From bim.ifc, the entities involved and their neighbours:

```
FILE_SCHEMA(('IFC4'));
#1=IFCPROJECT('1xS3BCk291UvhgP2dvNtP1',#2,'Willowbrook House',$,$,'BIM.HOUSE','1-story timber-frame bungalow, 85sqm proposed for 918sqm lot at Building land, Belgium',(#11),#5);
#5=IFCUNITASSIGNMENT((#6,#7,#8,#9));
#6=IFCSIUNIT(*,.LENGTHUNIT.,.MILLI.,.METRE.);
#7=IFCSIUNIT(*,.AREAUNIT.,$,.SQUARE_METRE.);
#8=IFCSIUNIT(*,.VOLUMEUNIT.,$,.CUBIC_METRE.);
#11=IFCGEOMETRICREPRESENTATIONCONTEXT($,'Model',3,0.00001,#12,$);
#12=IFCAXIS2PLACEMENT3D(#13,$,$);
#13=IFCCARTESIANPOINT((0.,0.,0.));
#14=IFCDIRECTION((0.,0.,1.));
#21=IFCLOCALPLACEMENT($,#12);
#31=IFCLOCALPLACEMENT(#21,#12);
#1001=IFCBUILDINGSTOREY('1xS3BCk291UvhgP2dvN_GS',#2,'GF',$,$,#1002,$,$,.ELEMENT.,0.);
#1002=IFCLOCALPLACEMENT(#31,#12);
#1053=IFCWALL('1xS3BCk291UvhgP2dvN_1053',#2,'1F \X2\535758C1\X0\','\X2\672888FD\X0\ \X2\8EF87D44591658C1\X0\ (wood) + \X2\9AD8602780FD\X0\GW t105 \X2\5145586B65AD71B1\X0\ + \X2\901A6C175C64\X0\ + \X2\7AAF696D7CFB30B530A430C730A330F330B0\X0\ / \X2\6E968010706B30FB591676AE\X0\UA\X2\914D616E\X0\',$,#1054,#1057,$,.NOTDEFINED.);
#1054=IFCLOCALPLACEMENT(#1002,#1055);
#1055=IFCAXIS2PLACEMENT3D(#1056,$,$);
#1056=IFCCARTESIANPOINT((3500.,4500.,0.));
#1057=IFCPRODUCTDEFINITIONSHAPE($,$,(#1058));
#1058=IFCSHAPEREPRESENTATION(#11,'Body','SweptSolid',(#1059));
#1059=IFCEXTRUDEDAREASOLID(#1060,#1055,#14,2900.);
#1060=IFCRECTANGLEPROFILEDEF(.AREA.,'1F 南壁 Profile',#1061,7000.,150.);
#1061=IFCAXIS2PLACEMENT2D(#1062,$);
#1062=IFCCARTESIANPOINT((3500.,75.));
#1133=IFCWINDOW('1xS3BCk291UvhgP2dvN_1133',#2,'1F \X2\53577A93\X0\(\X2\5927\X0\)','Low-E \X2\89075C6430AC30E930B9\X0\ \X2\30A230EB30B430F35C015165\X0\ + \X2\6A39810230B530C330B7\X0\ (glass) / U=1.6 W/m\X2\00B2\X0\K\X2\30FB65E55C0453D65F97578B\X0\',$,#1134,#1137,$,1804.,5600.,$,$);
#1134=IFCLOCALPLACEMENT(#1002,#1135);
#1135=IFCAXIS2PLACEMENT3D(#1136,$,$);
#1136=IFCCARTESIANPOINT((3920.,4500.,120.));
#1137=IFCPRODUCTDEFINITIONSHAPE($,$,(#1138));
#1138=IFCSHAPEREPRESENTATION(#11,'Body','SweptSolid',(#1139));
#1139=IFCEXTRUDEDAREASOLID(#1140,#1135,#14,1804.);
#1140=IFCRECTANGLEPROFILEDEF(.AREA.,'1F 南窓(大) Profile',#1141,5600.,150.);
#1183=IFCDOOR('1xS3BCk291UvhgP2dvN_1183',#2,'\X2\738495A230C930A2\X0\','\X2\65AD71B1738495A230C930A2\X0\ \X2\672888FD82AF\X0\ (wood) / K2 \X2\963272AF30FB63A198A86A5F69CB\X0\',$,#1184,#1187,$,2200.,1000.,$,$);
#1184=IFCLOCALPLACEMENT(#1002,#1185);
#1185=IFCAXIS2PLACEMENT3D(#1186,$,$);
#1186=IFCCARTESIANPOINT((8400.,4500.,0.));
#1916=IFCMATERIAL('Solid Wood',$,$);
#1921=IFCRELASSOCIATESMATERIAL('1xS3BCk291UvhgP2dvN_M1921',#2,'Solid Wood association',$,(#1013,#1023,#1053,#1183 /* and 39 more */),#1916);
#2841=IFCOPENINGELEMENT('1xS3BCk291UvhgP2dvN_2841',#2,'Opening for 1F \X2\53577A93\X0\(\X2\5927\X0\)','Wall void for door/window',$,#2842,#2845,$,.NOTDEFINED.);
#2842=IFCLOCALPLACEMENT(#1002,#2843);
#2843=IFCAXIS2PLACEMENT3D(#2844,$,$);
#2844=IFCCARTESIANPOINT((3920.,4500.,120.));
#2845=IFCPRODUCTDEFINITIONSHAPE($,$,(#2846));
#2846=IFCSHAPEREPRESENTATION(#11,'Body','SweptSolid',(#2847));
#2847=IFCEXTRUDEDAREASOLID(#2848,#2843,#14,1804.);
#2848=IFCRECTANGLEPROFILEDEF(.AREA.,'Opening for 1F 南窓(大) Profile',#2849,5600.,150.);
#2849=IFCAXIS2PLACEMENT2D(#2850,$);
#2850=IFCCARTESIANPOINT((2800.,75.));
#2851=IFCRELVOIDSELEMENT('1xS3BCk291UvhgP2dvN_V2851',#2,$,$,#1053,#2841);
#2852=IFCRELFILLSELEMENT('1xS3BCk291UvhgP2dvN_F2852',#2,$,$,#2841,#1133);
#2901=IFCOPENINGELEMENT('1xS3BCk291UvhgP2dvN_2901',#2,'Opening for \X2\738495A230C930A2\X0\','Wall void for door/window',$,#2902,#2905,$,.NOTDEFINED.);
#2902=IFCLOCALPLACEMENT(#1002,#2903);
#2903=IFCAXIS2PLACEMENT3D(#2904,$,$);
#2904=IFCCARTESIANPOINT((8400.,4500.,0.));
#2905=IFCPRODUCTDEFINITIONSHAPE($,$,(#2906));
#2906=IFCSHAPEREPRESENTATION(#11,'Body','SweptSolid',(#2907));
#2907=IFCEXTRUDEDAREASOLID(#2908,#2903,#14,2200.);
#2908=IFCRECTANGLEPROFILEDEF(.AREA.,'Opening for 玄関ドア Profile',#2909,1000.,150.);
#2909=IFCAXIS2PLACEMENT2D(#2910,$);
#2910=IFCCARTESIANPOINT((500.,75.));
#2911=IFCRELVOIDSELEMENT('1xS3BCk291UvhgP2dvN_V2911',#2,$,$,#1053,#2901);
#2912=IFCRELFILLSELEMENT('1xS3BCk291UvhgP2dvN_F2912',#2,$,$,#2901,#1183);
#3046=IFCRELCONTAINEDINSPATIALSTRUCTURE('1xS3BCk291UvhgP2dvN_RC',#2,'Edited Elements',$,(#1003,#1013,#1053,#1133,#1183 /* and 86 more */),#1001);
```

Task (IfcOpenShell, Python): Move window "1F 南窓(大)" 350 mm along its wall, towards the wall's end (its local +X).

```python
import ifcopenshell
import ifcopenshell.api.geometry
import ifcopenshell.util.placement
import ifcopenshell.util.unit

model = ifcopenshell.open("bim.ifc")
unit_scale = ifcopenshell.util.unit.calculate_unit_scale(model)

window = model.by_id(1133)
opening = window.FillsVoids[0].RelatingOpeningElement
wall = opening.VoidsElements[0].RelatingBuildingElement

wall_matrix = ifcopenshell.util.placement.get_local_placement(wall.ObjectPlacement)
shift = wall_matrix[:3, 0] * 0.35 / unit_scale
before = ifcopenshell.util.placement.get_local_placement(window.ObjectPlacement)[:3, 3].copy()

# The window is not placed relative to its opening, so move both.
for product in (opening, window):
    matrix = ifcopenshell.util.placement.get_local_placement(product.ObjectPlacement)
    matrix[:3, 3] += shift
    ifcopenshell.api.geometry.edit_object_placement(model, product=product, matrix=matrix, is_si=False)

after = ifcopenshell.util.placement.get_local_placement(window.ObjectPlacement)[:3, 3]
print("window moved by", (after - before).round(3) + 0.0)

model.write("bim_updated.ifc")
```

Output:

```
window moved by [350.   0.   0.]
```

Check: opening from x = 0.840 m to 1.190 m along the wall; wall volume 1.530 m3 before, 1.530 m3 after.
